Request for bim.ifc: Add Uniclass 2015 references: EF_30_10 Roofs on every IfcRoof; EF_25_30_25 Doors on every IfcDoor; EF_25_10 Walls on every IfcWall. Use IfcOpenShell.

First a look at what the model holds.

```python
import ifcopenshell

model = ifcopenshell.open("bim.ifc")
print(model.schema)
print("classifications:", [c.Name for c in model.by_type("IfcClassification")])
for ifc_class in ("IfcDoor", "IfcRoof", "IfcStair", "IfcWall", "IfcWindow"):
    print(ifc_class, len(model.by_type(ifc_class)))
```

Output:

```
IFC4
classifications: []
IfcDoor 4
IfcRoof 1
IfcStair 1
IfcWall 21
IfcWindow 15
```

```python
import ifcopenshell
import ifcopenshell.api.classification

model = ifcopenshell.open("bim.ifc")

system = ifcopenshell.api.classification.add_classification(model, classification="Uniclass 2015")

codes = {
    "IfcRoof": ("EF_30_10", "Roofs"),
    "IfcDoor": ("EF_25_30_25", "Doors"),
    "IfcWall": ("EF_25_10", "Walls"),
}
for ifc_class, (code, name) in codes.items():
    products = model.by_type(ifc_class)
    ifcopenshell.api.classification.add_reference(
        model, products=products, classification=system, identification=code, name=name
    )
    print(code, len(products))

model.write("bim_updated.ifc")
```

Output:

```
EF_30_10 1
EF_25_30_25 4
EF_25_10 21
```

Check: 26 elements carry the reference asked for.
